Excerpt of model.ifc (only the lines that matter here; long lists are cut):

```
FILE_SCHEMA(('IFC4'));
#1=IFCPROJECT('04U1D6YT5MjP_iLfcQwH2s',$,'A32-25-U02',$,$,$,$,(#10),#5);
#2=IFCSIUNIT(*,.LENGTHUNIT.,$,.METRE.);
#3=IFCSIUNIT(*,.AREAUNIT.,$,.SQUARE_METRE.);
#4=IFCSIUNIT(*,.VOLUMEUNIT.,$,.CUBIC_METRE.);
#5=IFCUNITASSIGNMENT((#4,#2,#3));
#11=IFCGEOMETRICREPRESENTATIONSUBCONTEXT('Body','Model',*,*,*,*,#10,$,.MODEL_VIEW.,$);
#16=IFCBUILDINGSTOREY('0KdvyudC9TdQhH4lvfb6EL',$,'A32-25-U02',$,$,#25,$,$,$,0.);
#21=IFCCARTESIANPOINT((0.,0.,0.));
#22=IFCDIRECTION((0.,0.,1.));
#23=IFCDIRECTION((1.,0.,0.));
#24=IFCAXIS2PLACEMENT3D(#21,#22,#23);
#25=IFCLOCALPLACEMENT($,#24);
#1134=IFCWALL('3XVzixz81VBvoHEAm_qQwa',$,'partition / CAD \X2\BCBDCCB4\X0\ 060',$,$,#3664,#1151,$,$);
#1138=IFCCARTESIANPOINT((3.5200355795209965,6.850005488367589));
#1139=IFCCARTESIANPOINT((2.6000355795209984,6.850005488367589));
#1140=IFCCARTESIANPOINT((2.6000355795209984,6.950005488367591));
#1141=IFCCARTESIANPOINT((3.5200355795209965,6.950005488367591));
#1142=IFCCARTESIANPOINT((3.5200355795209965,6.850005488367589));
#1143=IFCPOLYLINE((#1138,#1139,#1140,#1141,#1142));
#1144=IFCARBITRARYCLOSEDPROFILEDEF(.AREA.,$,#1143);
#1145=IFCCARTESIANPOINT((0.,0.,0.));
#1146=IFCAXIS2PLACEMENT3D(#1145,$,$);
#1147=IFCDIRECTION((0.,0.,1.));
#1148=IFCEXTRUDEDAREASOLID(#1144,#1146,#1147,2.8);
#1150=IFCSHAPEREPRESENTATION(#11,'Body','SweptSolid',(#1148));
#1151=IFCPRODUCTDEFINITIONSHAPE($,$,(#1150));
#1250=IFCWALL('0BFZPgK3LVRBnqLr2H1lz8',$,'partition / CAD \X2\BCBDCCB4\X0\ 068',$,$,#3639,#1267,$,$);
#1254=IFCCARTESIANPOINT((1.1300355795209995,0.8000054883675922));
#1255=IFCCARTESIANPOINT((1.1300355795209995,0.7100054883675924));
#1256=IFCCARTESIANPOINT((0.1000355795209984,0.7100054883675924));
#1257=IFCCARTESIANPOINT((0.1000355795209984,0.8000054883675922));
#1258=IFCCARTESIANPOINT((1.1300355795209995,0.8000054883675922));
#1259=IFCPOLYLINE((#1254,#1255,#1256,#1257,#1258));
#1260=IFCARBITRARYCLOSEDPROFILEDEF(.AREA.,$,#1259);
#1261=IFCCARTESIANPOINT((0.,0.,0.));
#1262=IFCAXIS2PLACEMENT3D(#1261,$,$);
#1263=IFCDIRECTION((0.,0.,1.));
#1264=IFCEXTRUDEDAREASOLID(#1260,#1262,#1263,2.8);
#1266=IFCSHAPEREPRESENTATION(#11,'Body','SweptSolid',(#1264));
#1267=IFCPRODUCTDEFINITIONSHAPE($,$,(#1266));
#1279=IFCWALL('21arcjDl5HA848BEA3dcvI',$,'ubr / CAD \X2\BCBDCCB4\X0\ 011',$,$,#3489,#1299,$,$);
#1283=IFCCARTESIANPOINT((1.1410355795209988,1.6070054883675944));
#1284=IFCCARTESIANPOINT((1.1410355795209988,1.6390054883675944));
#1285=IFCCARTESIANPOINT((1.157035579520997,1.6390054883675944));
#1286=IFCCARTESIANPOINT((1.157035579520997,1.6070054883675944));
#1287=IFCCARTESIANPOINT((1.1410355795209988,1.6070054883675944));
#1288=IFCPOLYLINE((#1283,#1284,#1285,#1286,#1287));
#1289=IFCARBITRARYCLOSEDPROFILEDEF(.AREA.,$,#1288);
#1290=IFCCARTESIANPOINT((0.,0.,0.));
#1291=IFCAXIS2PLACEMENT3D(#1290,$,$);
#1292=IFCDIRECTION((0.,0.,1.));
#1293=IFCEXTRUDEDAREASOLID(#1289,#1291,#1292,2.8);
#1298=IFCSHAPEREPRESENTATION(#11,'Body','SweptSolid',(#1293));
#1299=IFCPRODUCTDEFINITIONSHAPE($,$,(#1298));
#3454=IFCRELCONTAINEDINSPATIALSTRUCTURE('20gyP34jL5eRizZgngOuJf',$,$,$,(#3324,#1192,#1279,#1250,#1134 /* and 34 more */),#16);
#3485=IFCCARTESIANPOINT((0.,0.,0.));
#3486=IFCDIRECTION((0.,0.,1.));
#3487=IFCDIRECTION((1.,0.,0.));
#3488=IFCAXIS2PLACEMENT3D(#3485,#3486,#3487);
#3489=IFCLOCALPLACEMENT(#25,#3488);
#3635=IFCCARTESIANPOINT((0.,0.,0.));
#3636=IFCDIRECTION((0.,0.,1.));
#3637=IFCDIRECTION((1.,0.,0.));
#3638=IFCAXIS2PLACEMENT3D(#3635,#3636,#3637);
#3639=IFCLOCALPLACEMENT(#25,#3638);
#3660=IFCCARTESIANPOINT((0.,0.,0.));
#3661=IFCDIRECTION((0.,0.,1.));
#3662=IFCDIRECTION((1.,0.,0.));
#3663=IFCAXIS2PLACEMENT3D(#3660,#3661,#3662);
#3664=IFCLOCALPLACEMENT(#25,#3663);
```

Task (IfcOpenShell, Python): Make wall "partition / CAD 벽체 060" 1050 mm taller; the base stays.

```python
import ifcopenshell
import ifcopenshell.geom
import ifcopenshell.util.representation
import ifcopenshell.util.shape

model = ifcopenshell.open("model.ifc")
settings = ifcopenshell.geom.settings()


def volume(element):
    """Net volume in cubic metres, openings subtracted."""
    shape = ifcopenshell.geom.create_shape(settings, element)
    return ifcopenshell.util.shape.get_volume(shape.geometry)


wall = model.by_id(1134)
before = volume(wall)

body = ifcopenshell.util.representation.get_representation(wall, "Model", "Body")
solid = body.Items[0]
old_height = solid.Depth
solid.Depth += 1.05
after = volume(wall)

print(f"height {old_height:g} -> {solid.Depth:g}, volume {before:.3f} -> {after:.3f} m3")

model.write("model_updated.ifc")
```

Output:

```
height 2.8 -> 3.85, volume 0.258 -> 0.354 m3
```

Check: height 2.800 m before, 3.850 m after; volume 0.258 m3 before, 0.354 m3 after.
